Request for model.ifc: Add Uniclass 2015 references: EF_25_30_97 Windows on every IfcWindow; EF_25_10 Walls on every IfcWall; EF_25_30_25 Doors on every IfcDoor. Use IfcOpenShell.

First a look at what the model holds.

```python
import ifcopenshell

model = ifcopenshell.open("model.ifc")
print(model.schema)
print("classifications:", [c.Name for c in model.by_type("IfcClassification")])
for ifc_class in ("IfcDoor", "IfcRoof", "IfcStair", "IfcWall", "IfcWindow"):
    print(ifc_class, len(model.by_type(ifc_class)))
```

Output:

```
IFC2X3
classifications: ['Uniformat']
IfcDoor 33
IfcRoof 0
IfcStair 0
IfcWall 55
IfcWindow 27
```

```python
import ifcopenshell
import ifcopenshell.api.classification

model = ifcopenshell.open("model.ifc")

# IFC2X3 requires Source and Edition and has no link from the project to the system.
system = model.create_entity("IfcClassification", Source="NBS", Edition="2015", Name="Uniclass 2015")

codes = {
    "IfcWindow": ("EF_25_30_97", "Windows"),
    "IfcWall": ("EF_25_10", "Walls"),
    "IfcDoor": ("EF_25_30_25", "Doors"),
}
for ifc_class, (code, name) in codes.items():
    products = model.by_type(ifc_class)
    ifcopenshell.api.classification.add_reference(
        model, products=products, classification=system, identification=code, name=name
    )
    print(code, len(products))

model.write("model_v2.ifc")
```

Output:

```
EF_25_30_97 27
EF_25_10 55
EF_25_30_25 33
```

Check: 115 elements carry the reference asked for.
